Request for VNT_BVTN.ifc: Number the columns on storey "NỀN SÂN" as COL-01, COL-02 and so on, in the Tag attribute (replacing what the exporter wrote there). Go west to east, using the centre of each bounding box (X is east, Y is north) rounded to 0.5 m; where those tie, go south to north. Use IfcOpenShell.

First a look at what the model holds.

```python
import ifcopenshell
import ifcopenshell.util.element
import ifcopenshell.util.placement

model = ifcopenshell.open("VNT_BVTN.ifc")
print(model.schema)
storey = next(s for s in model.by_type("IfcBuildingStorey") if s.Name == "NỀN SÂN")
columns = [e for e in ifcopenshell.util.element.get_decomposition(storey) if e.is_a("IfcColumn")]
for e in sorted(columns, key=lambda e: e.id()):
    origin = ifcopenshell.util.placement.get_local_placement(e.ObjectPlacement)[:3, 3]
    print(e.id(), e.Tag, e.Name, origin.round(2) + 0.0, sep=" | ")
```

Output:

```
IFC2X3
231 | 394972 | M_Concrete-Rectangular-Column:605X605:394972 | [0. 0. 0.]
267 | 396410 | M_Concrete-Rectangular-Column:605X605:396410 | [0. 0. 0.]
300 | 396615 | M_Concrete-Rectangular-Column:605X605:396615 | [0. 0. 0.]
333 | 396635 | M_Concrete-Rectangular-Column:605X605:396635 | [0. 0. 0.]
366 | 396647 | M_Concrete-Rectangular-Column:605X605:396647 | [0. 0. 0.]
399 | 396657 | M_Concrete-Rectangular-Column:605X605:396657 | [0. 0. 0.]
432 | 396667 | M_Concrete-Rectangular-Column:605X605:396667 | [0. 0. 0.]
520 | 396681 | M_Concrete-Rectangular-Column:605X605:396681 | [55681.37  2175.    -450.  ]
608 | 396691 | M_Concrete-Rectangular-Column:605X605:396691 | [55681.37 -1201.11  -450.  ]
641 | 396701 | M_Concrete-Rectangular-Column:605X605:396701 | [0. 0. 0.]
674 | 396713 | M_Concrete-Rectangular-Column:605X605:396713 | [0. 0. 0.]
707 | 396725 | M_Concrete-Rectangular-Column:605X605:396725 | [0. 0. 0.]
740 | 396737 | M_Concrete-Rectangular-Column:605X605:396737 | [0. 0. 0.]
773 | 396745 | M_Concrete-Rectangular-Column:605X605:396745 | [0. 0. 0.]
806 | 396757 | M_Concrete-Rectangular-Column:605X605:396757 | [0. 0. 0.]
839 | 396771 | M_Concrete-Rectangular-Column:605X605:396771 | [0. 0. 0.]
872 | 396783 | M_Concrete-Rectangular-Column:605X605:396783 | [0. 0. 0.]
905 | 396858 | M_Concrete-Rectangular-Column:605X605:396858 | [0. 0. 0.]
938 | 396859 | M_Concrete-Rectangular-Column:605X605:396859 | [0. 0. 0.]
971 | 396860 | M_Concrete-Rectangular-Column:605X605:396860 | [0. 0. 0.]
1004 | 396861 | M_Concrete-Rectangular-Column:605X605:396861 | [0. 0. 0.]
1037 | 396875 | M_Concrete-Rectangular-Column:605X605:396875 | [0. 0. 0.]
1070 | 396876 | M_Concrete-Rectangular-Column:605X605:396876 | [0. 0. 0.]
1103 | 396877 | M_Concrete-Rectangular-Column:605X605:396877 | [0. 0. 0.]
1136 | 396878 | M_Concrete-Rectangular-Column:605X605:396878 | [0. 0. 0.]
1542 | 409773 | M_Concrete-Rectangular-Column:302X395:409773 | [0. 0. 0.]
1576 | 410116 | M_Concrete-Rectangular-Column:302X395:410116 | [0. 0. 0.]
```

```python
import ifcopenshell
import ifcopenshell.geom
import ifcopenshell.util.element
import ifcopenshell.util.shape

model = ifcopenshell.open("VNT_BVTN.ifc")
settings = ifcopenshell.geom.settings()
settings.set("use-world-coords", True)


def centre(element):
    shape = ifcopenshell.geom.create_shape(settings, element)
    return ifcopenshell.util.shape.get_bbox_centroid(shape.geometry)


storey = next(s for s in model.by_type("IfcBuildingStorey") if s.Name == "NỀN SÂN")
columns = [e for e in ifcopenshell.util.element.get_decomposition(storey) if e.is_a("IfcColumn")]

# Insertion points can sit at a corner or the storey origin, so sort by the geometry (in metres).
centres = {e: centre(e) for e in columns}
columns.sort(key=lambda e: (round(centres[e][0] / 0.5), centres[e][1]))

for i, e in enumerate(columns, start=1):
    number = f"COL-{i:02d}"
    e.Tag = number
    print(e.id(), number)

model.write("VNT_BVTN_edited.ifc")
```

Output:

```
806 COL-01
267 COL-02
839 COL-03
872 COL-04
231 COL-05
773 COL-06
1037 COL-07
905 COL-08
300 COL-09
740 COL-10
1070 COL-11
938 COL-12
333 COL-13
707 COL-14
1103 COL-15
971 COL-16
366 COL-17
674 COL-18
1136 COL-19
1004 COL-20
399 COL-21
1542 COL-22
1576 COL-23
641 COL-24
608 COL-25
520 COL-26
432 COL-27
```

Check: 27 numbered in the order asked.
